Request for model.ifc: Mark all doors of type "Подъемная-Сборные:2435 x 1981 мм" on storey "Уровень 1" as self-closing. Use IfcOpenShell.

First a look at what the model holds.

```python
import ifcopenshell
import ifcopenshell.util.element

model = ifcopenshell.open("model.ifc")
print(model.schema)
storey = next(s for s in model.by_type("IfcBuildingStorey") if s.Name == "Уровень 1")
doors = [e for e in ifcopenshell.util.element.get_decomposition(storey) if e.is_a("IfcDoor")]
seen = {}
for e in doors:
    element_type = ifcopenshell.util.element.get_type(e)
    key = (element_type.Name if element_type != e and element_type else None, ifcopenshell.util.element.get_pset(e, "Pset_DoorCommon", "SelfClosing"))
    seen[key] = seen.get(key, 0) + 1
for (name, value), count in sorted(seen.items(), key=str):
    print(count, "x", name, "|", value)
```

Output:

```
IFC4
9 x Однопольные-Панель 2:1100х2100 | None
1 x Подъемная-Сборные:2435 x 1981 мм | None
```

```python
import ifcopenshell
import ifcopenshell.api.pset
import ifcopenshell.util.element

model = ifcopenshell.open("model.ifc")

storey = next(s for s in model.by_type("IfcBuildingStorey") if s.Name == "Уровень 1")
doors = [e for e in ifcopenshell.util.element.get_decomposition(storey) if e.is_a("IfcDoor")]

count = 0
for e in doors:
    element_type = ifcopenshell.util.element.get_type(e)
    if element_type in (None, e) or element_type.Name != "Подъемная-Сборные:2435 x 1981 мм":
        continue
    # add_pset returns the element's existing set when there is one.
    pset = ifcopenshell.api.pset.add_pset(model, product=e, name="Pset_DoorCommon")
    ifcopenshell.api.pset.edit_pset(model, pset=pset, properties={"SelfClosing": True})
    count += 1

print(count, "doors updated")

model.write("model_rev.ifc")
```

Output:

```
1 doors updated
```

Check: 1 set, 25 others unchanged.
